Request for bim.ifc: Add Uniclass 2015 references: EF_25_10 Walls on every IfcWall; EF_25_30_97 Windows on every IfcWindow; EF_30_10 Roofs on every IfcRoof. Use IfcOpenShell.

First a look at what the model holds.

```python
import ifcopenshell

model = ifcopenshell.open("bim.ifc")
print(model.schema)
print("classifications:", [c.Name for c in model.by_type("IfcClassification")])
for ifc_class in ("IfcDoor", "IfcRoof", "IfcStair", "IfcWall", "IfcWindow"):
    print(ifc_class, len(model.by_type(ifc_class)))
```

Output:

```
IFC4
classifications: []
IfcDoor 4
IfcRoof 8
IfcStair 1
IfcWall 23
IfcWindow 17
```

```python
import ifcopenshell
import ifcopenshell.api.classification

model = ifcopenshell.open("bim.ifc")

system = ifcopenshell.api.classification.add_classification(model, classification="Uniclass 2015")

codes = {
    "IfcWall": ("EF_25_10", "Walls"),
    "IfcWindow": ("EF_25_30_97", "Windows"),
    "IfcRoof": ("EF_30_10", "Roofs"),
}
for ifc_class, (code, name) in codes.items():
    products = model.by_type(ifc_class)
    ifcopenshell.api.classification.add_reference(
        model, products=products, classification=system, identification=code, name=name
    )
    print(code, len(products))

model.write("bim_v2.ifc")
```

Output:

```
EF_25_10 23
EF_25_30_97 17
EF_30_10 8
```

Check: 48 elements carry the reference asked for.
